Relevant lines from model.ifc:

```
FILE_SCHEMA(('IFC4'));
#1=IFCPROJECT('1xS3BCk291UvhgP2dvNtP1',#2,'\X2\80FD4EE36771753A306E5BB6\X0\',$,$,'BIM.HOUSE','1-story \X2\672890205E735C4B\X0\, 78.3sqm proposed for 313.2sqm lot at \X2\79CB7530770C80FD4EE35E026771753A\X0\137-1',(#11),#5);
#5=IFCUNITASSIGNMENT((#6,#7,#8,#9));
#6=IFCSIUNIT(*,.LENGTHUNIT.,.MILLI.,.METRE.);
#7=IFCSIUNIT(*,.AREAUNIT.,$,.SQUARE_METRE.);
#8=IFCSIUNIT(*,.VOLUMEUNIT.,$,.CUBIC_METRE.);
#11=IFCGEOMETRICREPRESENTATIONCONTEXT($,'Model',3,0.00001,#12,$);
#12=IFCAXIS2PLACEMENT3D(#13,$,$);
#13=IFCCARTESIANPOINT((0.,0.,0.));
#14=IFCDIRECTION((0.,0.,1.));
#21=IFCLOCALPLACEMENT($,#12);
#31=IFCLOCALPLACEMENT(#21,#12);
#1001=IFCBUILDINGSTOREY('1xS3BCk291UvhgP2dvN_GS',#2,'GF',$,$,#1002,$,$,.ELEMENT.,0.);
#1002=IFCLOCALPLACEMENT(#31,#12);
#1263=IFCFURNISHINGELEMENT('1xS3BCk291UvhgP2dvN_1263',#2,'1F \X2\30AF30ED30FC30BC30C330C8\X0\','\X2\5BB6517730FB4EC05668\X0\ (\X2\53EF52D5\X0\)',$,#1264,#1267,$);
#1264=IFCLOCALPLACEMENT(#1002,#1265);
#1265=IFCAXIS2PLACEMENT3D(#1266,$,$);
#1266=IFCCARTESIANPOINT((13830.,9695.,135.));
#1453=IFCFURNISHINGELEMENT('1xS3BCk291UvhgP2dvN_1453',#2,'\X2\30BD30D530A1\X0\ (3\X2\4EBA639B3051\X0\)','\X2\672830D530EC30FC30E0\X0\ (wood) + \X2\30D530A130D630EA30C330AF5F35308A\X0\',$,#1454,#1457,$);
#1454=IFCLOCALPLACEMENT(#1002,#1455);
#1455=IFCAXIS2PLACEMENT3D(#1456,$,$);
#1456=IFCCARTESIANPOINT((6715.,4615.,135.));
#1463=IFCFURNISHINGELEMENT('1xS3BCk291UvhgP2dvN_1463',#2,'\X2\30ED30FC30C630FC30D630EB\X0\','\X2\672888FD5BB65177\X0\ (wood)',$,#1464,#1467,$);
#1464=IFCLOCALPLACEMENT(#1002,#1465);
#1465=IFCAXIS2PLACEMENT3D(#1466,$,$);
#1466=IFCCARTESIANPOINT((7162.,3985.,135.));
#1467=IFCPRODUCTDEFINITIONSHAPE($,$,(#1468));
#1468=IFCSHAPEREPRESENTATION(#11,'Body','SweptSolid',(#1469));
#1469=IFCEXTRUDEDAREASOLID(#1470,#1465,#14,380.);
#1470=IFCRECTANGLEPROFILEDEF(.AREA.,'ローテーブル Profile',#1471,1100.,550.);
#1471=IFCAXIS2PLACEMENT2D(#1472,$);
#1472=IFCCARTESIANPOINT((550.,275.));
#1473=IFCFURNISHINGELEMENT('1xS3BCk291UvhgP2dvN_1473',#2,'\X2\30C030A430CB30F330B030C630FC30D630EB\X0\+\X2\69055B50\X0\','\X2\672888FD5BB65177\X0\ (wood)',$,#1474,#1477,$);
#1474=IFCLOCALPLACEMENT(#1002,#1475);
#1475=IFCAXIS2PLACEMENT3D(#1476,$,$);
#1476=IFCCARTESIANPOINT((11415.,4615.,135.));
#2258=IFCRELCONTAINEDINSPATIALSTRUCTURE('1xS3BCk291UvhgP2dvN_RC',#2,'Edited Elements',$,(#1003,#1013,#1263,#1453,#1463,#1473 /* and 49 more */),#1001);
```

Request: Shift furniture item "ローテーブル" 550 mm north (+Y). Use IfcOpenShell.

```python
import ifcopenshell
import ifcopenshell.api.geometry
import ifcopenshell.util.placement

model = ifcopenshell.open("model.ifc")

item = model.by_guid("1xS3BCk291UvhgP2dvN_1463")
matrix = ifcopenshell.util.placement.get_local_placement(item.ObjectPlacement)
matrix[1, 3] += 550.0
ifcopenshell.api.geometry.edit_object_placement(model, product=item, matrix=matrix, is_si=False)

print(ifcopenshell.util.placement.get_local_placement(item.ObjectPlacement).round(3) + 0.0)

model.write("model_v2.ifc")
```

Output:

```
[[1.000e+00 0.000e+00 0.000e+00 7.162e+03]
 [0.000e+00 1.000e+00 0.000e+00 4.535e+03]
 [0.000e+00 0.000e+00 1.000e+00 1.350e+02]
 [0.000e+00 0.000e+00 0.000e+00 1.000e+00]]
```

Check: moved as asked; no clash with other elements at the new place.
